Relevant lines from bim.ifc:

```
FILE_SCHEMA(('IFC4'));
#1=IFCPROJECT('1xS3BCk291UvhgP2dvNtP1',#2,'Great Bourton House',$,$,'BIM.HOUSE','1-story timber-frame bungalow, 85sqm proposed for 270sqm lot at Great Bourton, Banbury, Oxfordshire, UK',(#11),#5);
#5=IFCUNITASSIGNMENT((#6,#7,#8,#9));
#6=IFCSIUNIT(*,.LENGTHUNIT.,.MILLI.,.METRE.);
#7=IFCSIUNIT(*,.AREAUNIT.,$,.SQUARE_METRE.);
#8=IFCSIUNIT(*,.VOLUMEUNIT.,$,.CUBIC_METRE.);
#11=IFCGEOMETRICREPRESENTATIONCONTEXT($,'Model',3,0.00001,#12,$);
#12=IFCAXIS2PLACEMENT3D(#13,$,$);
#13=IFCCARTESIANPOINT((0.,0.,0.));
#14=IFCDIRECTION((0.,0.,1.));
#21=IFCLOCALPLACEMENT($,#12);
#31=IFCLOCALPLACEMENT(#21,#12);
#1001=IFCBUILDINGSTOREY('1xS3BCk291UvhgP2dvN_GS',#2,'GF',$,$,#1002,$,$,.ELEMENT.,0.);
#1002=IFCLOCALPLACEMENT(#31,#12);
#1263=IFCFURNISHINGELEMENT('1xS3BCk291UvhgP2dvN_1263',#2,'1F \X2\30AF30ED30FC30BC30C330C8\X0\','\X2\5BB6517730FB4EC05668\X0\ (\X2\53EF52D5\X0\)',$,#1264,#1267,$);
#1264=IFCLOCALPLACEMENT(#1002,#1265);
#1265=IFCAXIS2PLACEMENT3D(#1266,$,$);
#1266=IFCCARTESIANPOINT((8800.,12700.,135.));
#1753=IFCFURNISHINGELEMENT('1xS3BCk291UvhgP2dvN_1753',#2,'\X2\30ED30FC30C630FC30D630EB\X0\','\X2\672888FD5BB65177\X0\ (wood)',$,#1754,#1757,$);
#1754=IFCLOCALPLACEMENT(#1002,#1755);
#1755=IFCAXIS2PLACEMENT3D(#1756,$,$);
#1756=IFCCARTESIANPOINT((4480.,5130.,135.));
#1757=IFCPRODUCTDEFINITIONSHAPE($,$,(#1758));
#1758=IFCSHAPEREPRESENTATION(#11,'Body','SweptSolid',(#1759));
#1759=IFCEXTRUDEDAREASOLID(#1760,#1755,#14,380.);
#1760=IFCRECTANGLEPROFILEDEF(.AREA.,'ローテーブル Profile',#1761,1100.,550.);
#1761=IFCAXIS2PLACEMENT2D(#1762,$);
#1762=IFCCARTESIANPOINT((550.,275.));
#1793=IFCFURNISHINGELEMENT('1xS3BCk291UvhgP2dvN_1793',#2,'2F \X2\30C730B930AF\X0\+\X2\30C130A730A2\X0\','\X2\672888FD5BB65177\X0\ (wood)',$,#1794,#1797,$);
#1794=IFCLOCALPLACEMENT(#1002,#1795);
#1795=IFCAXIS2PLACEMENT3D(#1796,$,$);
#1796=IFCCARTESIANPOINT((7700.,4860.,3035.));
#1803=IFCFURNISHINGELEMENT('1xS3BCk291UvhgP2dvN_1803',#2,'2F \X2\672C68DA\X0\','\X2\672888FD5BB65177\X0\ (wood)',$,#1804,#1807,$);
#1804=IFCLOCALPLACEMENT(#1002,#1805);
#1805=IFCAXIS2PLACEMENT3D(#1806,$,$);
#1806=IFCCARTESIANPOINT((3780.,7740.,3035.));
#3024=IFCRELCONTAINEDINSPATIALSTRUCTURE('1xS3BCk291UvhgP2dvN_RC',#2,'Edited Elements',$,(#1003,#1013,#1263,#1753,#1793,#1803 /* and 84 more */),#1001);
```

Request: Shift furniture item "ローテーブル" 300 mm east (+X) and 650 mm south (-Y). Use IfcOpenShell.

```python
import ifcopenshell
import ifcopenshell.api.geometry
import ifcopenshell.util.placement

model = ifcopenshell.open("bim.ifc")

item = model.by_guid("1xS3BCk291UvhgP2dvN_1753")
matrix = ifcopenshell.util.placement.get_local_placement(item.ObjectPlacement)
matrix[0, 3] += 300.0
matrix[1, 3] -= 650.0
ifcopenshell.api.geometry.edit_object_placement(model, product=item, matrix=matrix, is_si=False)

print(ifcopenshell.util.placement.get_local_placement(item.ObjectPlacement).round(3) + 0.0)

model.write("bim_updated.ifc")
```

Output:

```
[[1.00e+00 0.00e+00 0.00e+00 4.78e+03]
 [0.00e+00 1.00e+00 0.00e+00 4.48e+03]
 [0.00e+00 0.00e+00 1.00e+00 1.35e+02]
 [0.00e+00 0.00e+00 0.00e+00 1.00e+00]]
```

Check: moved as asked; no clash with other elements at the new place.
